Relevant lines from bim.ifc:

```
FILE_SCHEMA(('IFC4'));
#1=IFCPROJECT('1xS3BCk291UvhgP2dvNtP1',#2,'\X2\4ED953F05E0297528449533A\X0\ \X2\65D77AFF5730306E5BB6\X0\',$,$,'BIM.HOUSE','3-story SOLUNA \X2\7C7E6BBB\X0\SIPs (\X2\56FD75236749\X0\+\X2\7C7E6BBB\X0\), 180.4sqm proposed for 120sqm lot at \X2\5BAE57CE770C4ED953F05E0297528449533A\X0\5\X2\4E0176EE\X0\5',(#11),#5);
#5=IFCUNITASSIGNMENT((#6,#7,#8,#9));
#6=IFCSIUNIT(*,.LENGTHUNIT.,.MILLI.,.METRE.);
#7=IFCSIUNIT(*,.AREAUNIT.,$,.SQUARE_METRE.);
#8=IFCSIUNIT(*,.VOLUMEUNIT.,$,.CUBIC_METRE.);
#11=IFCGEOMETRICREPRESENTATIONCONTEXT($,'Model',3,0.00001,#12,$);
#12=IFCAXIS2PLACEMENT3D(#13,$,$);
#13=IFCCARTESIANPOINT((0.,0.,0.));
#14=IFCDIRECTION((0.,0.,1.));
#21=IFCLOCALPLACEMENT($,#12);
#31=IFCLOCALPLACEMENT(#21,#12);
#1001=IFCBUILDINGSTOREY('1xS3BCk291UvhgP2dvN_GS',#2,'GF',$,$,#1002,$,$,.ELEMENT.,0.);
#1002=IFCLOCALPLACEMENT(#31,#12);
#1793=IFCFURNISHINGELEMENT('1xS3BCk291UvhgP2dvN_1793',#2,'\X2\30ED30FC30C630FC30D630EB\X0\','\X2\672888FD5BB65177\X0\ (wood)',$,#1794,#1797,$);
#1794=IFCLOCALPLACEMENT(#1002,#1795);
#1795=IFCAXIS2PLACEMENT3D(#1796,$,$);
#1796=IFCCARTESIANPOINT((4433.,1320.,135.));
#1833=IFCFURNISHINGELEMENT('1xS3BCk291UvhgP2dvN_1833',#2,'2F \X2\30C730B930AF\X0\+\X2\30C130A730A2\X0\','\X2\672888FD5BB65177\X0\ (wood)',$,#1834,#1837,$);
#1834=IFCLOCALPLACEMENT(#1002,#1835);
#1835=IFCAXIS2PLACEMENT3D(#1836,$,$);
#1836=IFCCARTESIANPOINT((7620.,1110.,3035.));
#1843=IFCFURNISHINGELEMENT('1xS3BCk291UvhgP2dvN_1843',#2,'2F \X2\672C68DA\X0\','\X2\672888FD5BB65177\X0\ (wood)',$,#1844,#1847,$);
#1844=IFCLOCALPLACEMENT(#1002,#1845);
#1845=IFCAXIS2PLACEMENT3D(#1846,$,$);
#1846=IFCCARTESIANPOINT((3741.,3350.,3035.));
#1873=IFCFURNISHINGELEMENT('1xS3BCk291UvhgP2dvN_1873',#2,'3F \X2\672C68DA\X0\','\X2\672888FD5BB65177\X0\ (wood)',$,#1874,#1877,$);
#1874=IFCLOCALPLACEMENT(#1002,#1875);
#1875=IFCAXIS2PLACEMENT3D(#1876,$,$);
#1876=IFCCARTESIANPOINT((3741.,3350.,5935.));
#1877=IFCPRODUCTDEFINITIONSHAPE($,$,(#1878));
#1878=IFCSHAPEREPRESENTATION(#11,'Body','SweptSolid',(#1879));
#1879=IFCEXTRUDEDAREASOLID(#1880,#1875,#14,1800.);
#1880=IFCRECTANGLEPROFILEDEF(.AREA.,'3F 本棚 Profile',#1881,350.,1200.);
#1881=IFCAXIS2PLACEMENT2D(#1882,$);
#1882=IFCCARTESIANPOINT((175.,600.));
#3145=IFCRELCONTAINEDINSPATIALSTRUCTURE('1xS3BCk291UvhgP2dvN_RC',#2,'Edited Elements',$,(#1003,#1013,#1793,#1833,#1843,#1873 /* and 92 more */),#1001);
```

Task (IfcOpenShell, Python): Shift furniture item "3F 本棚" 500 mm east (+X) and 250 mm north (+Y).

```python
import ifcopenshell
import ifcopenshell.api.geometry
import ifcopenshell.util.placement
import ifcopenshell.util.unit

model = ifcopenshell.open("bim.ifc")
unit_scale = ifcopenshell.util.unit.calculate_unit_scale(model)

item = model.by_id(1873)
matrix = ifcopenshell.util.placement.get_local_placement(item.ObjectPlacement)
matrix[0, 3] += 0.5 / unit_scale
matrix[1, 3] += 0.25 / unit_scale
ifcopenshell.api.geometry.edit_object_placement(model, product=item, matrix=matrix, is_si=False)

print(ifcopenshell.util.placement.get_local_placement(item.ObjectPlacement).round(3) + 0.0)

model.write("bim_v2.ifc")
```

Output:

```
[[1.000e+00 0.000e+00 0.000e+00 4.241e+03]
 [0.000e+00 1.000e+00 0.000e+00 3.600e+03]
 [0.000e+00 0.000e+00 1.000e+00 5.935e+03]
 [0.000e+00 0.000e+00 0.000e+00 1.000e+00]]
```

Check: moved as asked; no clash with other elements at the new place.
